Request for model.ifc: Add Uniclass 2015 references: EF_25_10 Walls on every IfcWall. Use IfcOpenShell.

First a look at what the model holds.

```python
import ifcopenshell

model = ifcopenshell.open("model.ifc")
print(model.schema)
print("classifications:", [c.Name for c in model.by_type("IfcClassification")])
for ifc_class in ("IfcDoor", "IfcRoof", "IfcStair", "IfcWall", "IfcWindow"):
    print(ifc_class, len(model.by_type(ifc_class)))
```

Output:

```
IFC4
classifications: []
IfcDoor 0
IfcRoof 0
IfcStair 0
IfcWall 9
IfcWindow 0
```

```python
import ifcopenshell
import ifcopenshell.api.classification

model = ifcopenshell.open("model.ifc")

system = ifcopenshell.api.classification.add_classification(model, classification="Uniclass 2015")

codes = {
    "IfcWall": ("EF_25_10", "Walls"),
}
for ifc_class, (code, name) in codes.items():
    products = model.by_type(ifc_class)
    ifcopenshell.api.classification.add_reference(
        model, products=products, classification=system, identification=code, name=name
    )
    print(code, len(products))

model.write("model_v2.ifc")
```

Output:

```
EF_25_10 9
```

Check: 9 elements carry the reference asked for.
